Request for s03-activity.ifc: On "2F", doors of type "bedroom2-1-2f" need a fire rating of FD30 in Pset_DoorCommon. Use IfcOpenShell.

First a look at what the model holds.

```python
import ifcopenshell
import ifcopenshell.util.element

model = ifcopenshell.open("s03-activity.ifc")
print(model.schema)
storey = next(s for s in model.by_type("IfcBuildingStorey") if s.Name == "2F")
doors = [e for e in ifcopenshell.util.element.get_decomposition(storey) if e.is_a("IfcDoor")]
seen = {}
for e in doors:
    element_type = ifcopenshell.util.element.get_type(e)
    key = (element_type.Name if element_type != e and element_type else None, ifcopenshell.util.element.get_pset(e, "Pset_DoorCommon", "FireRating"))
    seen[key] = seen.get(key, 0) + 1
for (name, value), count in sorted(seen.items(), key=str):
    print(count, "x", name, "|", value)
```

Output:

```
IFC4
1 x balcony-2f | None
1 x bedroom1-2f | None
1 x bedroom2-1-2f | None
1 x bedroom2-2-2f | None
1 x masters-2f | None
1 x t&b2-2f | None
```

```python
import ifcopenshell
import ifcopenshell.api.pset
import ifcopenshell.util.element

model = ifcopenshell.open("s03-activity.ifc")

storey = next(s for s in model.by_type("IfcBuildingStorey") if s.Name == "2F")
doors = [e for e in ifcopenshell.util.element.get_decomposition(storey) if e.is_a("IfcDoor")]

count = 0
for e in doors:
    element_type = ifcopenshell.util.element.get_type(e)
    if element_type in (None, e) or element_type.Name != "bedroom2-1-2f":
        continue
    # add_pset returns the element's existing set when there is one.
    pset = ifcopenshell.api.pset.add_pset(model, product=e, name="Pset_DoorCommon")
    ifcopenshell.api.pset.edit_pset(model, pset=pset, properties={"FireRating": "FD30"})
    count += 1

print(count, "doors updated")

model.write("s03-activity-out.ifc")
```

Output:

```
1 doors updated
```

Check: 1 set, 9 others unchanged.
